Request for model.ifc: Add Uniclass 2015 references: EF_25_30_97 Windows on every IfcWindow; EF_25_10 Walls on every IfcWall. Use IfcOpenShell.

First a look at what the model holds.

```python
import ifcopenshell

model = ifcopenshell.open("model.ifc")
print(model.schema)
print("classifications:", [c.Name for c in model.by_type("IfcClassification")])
for ifc_class in ("IfcDoor", "IfcRoof", "IfcStair", "IfcWall", "IfcWindow"):
    print(ifc_class, len(model.by_type(ifc_class)))
```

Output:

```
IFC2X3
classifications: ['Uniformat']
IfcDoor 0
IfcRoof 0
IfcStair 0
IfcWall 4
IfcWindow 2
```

```python
import ifcopenshell
import ifcopenshell.api.classification

model = ifcopenshell.open("model.ifc")

# IFC2X3 requires Source and Edition and has no link from the project to the system.
system = model.create_entity("IfcClassification", Source="NBS", Edition="2015", Name="Uniclass 2015")

codes = {
    "IfcWindow": ("EF_25_30_97", "Windows"),
    "IfcWall": ("EF_25_10", "Walls"),
}
for ifc_class, (code, name) in codes.items():
    products = model.by_type(ifc_class)
    ifcopenshell.api.classification.add_reference(
        model, products=products, classification=system, identification=code, name=name
    )
    print(code, len(products))

model.write("model_updated.ifc")
```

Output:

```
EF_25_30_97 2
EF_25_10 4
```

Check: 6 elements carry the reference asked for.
